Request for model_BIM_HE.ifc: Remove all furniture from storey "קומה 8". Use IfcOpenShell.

First a look at what the model holds.

```python
import ifcopenshell
import ifcopenshell.util.element

model = ifcopenshell.open("model_BIM_HE.ifc")
print(model.schema)
storey = next(s for s in model.by_type("IfcBuildingStorey") if s.Name == "קומה 8")
furniture = [e for e in ifcopenshell.util.element.get_decomposition(storey) if e.is_a("IfcFurnishingElement")]
seen = {}
for e in furniture:
    element_type = ifcopenshell.util.element.get_type(e)
    name = element_type.Name if element_type not in (None, e) else None
    seen[name] = seen.get(name, 0) + 1
for name, count in sorted(seen.items(), key=str):
    print(count, "x", name)
```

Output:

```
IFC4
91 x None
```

```python
import ifcopenshell
import ifcopenshell.api.root
import ifcopenshell.util.element

model = ifcopenshell.open("model_BIM_HE.ifc")

storey = next(s for s in model.by_type("IfcBuildingStorey") if s.Name == "קומה 8")
furniture = [e for e in ifcopenshell.util.element.get_decomposition(storey) if e.is_a("IfcFurnishingElement")]

for e in furniture:
    ifcopenshell.api.root.remove_product(model, product=e)
print(len(furniture), "removed")

model.write("model_BIM_HE_edited.ifc")
```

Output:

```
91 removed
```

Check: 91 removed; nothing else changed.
